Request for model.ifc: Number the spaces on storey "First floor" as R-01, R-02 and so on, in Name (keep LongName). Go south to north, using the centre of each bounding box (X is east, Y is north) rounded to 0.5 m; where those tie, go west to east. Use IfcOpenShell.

First a look at what the model holds.

```python
import ifcopenshell
import ifcopenshell.util.element
import ifcopenshell.util.placement

model = ifcopenshell.open("model.ifc")
print(model.schema)
storey = next(s for s in model.by_type("IfcBuildingStorey") if s.Name == "First floor")
spaces = [e for e in ifcopenshell.util.element.get_decomposition(storey) if e.is_a("IfcSpace")]
for e in sorted(spaces, key=lambda e: e.id()):
    origin = ifcopenshell.util.placement.get_local_placement(e.ObjectPlacement)[:3, 3]
    print(e.id(), e.Name, e.LongName, origin.round(2) + 0.0, sep=" | ")
```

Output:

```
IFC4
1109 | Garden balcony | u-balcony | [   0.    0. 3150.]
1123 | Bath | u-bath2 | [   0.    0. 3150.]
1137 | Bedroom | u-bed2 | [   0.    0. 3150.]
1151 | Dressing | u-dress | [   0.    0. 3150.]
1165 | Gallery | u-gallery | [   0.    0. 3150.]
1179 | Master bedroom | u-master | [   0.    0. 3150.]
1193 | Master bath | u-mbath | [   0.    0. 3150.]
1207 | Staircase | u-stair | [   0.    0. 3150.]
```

```python
import ifcopenshell
import ifcopenshell.geom
import ifcopenshell.util.element
import ifcopenshell.util.shape

model = ifcopenshell.open("model.ifc")
settings = ifcopenshell.geom.settings()
settings.set("use-world-coords", True)


def centre(element):
    shape = ifcopenshell.geom.create_shape(settings, element)
    return ifcopenshell.util.shape.get_bbox_centroid(shape.geometry)


storey = next(s for s in model.by_type("IfcBuildingStorey") if s.Name == "First floor")
spaces = [e for e in ifcopenshell.util.element.get_decomposition(storey) if e.is_a("IfcSpace")]

# Insertion points can sit at a corner or the storey origin, so sort by the geometry (in metres).
centres = {e: centre(e) for e in spaces}
spaces.sort(key=lambda e: (round(centres[e][1] / 0.5), centres[e][0]))

for i, e in enumerate(spaces, start=1):
    number = f"R-{i:02d}"
    e.Name = number
    print(e.id(), number)

model.write("model_rev.ifc")
```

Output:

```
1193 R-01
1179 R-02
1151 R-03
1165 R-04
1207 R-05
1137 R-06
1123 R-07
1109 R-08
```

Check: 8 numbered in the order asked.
